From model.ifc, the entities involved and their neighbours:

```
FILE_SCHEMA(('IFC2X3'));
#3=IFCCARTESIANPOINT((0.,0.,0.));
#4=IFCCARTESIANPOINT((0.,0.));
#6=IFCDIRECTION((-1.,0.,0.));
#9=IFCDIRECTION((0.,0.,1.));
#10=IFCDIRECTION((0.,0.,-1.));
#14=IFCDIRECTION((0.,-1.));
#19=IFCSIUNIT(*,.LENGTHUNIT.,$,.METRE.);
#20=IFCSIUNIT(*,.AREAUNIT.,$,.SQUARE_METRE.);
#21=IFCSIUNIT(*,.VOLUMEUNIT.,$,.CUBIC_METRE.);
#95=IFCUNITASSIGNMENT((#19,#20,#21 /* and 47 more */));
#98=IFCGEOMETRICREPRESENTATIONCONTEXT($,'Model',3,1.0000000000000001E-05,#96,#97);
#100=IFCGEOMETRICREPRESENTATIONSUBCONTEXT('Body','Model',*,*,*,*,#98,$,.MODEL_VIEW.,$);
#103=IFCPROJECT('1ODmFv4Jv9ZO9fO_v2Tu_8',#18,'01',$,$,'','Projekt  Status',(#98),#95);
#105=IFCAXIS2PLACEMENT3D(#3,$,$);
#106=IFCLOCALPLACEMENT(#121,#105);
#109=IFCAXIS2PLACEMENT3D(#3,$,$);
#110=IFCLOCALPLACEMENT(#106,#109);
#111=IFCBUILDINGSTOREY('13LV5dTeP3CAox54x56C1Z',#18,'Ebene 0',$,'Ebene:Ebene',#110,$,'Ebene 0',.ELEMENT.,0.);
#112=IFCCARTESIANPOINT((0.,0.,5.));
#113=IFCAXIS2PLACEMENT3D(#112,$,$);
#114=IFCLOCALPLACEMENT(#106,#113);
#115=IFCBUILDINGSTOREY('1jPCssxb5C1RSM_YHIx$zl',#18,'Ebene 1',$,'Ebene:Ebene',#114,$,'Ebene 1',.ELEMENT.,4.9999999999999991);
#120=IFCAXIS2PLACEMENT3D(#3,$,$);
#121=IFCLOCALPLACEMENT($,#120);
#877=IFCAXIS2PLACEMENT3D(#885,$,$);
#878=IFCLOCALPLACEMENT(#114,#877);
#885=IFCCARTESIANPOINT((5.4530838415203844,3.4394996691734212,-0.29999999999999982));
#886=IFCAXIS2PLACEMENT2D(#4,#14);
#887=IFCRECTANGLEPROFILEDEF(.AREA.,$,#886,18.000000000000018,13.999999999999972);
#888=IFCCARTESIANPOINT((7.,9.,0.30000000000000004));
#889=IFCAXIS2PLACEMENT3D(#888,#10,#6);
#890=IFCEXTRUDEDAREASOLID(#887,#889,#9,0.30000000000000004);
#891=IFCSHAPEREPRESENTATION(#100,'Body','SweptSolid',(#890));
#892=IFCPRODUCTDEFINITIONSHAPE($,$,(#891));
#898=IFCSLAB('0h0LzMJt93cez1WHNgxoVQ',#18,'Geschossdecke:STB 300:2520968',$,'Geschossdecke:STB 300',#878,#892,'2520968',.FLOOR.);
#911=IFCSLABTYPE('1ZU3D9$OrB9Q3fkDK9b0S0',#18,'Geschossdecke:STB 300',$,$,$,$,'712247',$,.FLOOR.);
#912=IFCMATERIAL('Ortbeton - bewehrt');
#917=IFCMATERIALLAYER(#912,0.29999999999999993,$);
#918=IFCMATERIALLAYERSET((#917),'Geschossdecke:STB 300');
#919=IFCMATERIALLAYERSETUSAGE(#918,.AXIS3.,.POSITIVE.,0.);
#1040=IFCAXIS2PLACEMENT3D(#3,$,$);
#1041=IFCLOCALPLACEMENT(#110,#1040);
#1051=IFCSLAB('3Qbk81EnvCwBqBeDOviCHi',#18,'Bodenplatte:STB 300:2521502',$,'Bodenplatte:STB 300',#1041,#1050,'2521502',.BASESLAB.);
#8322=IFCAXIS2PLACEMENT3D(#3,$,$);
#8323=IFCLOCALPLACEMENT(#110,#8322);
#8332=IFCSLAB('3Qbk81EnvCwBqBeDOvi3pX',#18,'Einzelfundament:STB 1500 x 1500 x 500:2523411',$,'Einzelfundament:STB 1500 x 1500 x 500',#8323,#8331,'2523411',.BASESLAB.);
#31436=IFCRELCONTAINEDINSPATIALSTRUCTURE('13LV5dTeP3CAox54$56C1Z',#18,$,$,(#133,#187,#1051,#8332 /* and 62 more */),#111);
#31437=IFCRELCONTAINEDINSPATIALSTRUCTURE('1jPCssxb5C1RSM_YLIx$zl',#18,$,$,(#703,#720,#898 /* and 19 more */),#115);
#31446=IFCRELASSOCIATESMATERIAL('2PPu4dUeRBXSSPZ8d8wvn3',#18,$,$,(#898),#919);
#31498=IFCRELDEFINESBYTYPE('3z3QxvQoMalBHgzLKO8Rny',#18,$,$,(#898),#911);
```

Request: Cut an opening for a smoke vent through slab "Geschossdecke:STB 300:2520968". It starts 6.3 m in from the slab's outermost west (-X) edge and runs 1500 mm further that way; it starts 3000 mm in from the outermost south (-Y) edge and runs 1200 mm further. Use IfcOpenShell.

```python
import numpy as np
import ifcopenshell
import ifcopenshell.api.feature
import ifcopenshell.api.geometry
import ifcopenshell.api.root
import ifcopenshell.geom
import ifcopenshell.util.placement
import ifcopenshell.util.representation
import ifcopenshell.util.shape
import ifcopenshell.util.unit

model = ifcopenshell.open("model.ifc")
unit_scale = ifcopenshell.util.unit.calculate_unit_scale(model)
settings = ifcopenshell.geom.settings()


def volume(element):
    """Net volume in cubic metres, openings subtracted."""
    shape = ifcopenshell.geom.create_shape(settings, element)
    return ifcopenshell.util.shape.get_volume(shape.geometry)


slab = model.by_id(898)
before = volume(slab)

# Extent in the slab's own axes, in metres. The edges named are its -X and -Y sides.
slab_shape = ifcopenshell.geom.create_shape(settings, slab)
vertices = ifcopenshell.util.shape.get_vertices(slab_shape.geometry)
x_min, y_min, bottom = vertices.min(axis=0)
top = vertices[:, 2].max()

opening = ifcopenshell.api.root.create_entity(model, ifc_class="IfcOpeningElement", name="Smoke vent opening")
context = ifcopenshell.util.representation.get_context(model, "Model", "Body", "MODEL_VIEW")
width, depth = 1.5, 1.2
outline = [(0.0, 0.0), (width, 0.0), (width, depth), (0.0, depth), (0.0, 0.0)]
# Overshoot both faces by 50 mm so the cut is clean.
shape = ifcopenshell.api.geometry.add_slab_representation(
    model, context=context, depth=top - bottom + 0.1, polyline=outline
)
ifcopenshell.api.geometry.assign_representation(model, product=opening, representation=shape)

matrix = ifcopenshell.util.placement.get_local_placement(slab.ObjectPlacement)
matrix[:, 3] = matrix @ np.append(np.array([x_min + 6.3, y_min + 3, bottom - 0.05]) / unit_scale, 1.0)
ifcopenshell.api.geometry.edit_object_placement(model, product=opening, matrix=matrix, is_si=False)
ifcopenshell.api.feature.add_feature(model, feature=opening, element=slab)

after = volume(slab)

print(f"slab volume {before:.3f} -> {after:.3f} m3")

model.write("model_rev.ifc")
```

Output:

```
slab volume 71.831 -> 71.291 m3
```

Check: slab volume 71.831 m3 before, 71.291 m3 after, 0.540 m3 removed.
